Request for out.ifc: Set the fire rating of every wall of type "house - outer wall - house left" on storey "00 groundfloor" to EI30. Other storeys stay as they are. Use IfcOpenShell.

First a look at what the model holds.

```python
import ifcopenshell
import ifcopenshell.util.element

model = ifcopenshell.open("out.ifc")
print(model.schema)
storey = next(s for s in model.by_type("IfcBuildingStorey") if s.Name == "00 groundfloor")
walls = [e for e in ifcopenshell.util.element.get_decomposition(storey) if e.is_a("IfcWall")]
seen = {}
for e in walls:
    element_type = ifcopenshell.util.element.get_type(e)
    key = (element_type.Name if element_type != e and element_type else None, ifcopenshell.util.element.get_pset(e, "Pset_WallCommon", "FireRating"))
    seen[key] = seen.get(key, 0) + 1
for (name, value), count in sorted(seen.items(), key=str):
    print(count, "x", name, "|", value)
```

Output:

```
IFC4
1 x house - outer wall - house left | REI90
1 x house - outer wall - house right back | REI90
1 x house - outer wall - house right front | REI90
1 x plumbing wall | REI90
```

```python
import ifcopenshell
import ifcopenshell.api.pset
import ifcopenshell.util.element

model = ifcopenshell.open("out.ifc")

storey = next(s for s in model.by_type("IfcBuildingStorey") if s.Name == "00 groundfloor")
walls = [e for e in ifcopenshell.util.element.get_decomposition(storey) if e.is_a("IfcWall")]

count = 0
for e in walls:
    element_type = ifcopenshell.util.element.get_type(e)
    if element_type in (None, e) or element_type.Name != "house - outer wall - house left":
        continue
    # add_pset returns the element's existing set when there is one.
    pset = ifcopenshell.api.pset.add_pset(model, product=e, name="Pset_WallCommon")
    ifcopenshell.api.pset.edit_pset(model, pset=pset, properties={"FireRating": "EI30"})
    count += 1

print(count, "walls updated")

model.write("out_updated.ifc")
```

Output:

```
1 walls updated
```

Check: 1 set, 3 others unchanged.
